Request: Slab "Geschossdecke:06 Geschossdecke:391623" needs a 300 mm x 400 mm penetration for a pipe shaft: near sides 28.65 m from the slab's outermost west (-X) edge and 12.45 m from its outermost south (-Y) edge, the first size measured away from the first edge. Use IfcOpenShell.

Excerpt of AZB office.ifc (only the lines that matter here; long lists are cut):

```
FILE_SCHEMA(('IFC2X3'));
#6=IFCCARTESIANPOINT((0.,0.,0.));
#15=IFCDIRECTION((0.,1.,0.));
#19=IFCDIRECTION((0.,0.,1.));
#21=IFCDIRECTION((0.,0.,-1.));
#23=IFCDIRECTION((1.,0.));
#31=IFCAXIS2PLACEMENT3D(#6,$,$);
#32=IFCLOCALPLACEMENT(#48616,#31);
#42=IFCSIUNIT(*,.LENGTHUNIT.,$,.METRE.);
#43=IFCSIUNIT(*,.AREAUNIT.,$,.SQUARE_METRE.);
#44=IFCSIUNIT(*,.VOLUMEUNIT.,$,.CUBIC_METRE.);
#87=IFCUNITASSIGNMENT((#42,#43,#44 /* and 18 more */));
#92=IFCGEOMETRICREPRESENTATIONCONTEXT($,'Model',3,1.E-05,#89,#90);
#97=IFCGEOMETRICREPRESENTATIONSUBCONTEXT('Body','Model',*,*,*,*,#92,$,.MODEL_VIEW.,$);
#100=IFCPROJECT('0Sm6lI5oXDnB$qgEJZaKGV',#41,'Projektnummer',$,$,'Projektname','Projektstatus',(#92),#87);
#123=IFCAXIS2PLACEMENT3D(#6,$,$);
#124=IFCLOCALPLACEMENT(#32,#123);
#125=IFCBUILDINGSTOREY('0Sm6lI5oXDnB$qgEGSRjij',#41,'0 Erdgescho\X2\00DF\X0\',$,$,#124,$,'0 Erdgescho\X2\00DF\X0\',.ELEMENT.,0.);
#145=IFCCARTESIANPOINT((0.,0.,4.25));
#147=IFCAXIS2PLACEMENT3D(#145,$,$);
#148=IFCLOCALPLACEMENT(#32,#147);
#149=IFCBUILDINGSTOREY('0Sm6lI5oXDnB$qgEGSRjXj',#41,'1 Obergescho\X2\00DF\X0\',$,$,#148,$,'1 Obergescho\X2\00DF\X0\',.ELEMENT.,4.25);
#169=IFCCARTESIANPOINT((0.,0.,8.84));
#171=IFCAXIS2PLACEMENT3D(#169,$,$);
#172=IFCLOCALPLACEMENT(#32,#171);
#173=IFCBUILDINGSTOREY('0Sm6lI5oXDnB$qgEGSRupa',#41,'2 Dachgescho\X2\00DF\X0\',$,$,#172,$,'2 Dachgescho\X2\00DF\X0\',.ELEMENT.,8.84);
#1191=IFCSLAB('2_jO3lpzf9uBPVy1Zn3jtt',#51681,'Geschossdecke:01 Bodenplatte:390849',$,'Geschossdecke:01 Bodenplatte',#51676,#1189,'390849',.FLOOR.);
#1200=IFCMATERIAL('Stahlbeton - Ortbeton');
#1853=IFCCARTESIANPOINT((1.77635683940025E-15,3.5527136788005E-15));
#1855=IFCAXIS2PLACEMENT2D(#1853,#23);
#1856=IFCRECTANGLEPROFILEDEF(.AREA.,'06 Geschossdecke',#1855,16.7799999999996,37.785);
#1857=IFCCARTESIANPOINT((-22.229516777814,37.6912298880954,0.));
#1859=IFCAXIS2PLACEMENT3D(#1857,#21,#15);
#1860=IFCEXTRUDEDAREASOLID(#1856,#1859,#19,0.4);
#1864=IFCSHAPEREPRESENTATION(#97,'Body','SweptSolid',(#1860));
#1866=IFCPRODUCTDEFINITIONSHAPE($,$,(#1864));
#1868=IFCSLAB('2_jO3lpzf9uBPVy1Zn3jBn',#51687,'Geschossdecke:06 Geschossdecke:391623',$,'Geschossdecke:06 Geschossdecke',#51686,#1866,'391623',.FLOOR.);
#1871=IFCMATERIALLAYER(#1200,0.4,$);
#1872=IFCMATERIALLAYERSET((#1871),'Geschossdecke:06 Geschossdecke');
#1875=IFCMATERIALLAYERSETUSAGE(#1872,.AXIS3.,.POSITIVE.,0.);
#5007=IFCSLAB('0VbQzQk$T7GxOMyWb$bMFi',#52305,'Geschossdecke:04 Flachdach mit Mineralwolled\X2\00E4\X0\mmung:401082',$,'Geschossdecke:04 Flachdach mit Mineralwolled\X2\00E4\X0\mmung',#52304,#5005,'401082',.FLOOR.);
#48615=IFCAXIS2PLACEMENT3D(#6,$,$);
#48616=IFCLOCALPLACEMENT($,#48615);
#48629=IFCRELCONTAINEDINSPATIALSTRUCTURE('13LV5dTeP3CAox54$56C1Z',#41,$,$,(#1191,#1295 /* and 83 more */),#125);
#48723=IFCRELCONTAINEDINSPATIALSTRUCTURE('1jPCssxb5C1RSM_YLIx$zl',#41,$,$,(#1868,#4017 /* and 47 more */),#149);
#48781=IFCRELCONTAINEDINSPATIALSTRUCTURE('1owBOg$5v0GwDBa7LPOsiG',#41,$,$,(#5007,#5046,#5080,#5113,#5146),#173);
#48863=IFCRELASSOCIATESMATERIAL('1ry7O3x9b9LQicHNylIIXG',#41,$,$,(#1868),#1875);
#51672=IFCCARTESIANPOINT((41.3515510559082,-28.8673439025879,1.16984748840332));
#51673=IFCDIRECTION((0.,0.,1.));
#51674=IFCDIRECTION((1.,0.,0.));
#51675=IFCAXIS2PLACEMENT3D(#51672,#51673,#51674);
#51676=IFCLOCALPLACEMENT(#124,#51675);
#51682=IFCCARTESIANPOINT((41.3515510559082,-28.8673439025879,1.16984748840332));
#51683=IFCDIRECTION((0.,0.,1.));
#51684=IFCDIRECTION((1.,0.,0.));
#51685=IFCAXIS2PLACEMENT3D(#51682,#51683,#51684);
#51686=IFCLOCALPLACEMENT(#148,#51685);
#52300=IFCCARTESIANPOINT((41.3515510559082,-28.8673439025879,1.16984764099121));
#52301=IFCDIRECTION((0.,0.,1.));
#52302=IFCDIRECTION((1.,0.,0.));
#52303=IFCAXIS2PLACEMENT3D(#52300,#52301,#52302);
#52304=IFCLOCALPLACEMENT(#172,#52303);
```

```python
import numpy as np
import ifcopenshell
import ifcopenshell.api.feature
import ifcopenshell.api.geometry
import ifcopenshell.api.root
import ifcopenshell.geom
import ifcopenshell.util.placement
import ifcopenshell.util.representation
import ifcopenshell.util.shape
import ifcopenshell.util.unit

model = ifcopenshell.open("AZB office.ifc")
unit_scale = ifcopenshell.util.unit.calculate_unit_scale(model)
settings = ifcopenshell.geom.settings()


def volume(element):
    """Net volume in cubic metres, openings subtracted."""
    shape = ifcopenshell.geom.create_shape(settings, element)
    return ifcopenshell.util.shape.get_volume(shape.geometry)


slab = model.by_guid("2_jO3lpzf9uBPVy1Zn3jBn")
before = volume(slab)

# Extent in the slab's own axes, in metres. The edges named are its -X and -Y sides.
slab_shape = ifcopenshell.geom.create_shape(settings, slab)
vertices = ifcopenshell.util.shape.get_vertices(slab_shape.geometry)
x_min, y_min, bottom = vertices.min(axis=0)
top = vertices[:, 2].max()

opening = ifcopenshell.api.root.create_entity(model, ifc_class="IfcOpeningElement", name="Pipe shaft opening")
context = ifcopenshell.util.representation.get_context(model, "Model", "Body", "MODEL_VIEW")
width, depth = 0.3, 0.4
outline = [(0.0, 0.0), (width, 0.0), (width, depth), (0.0, depth), (0.0, 0.0)]
# Overshoot both faces by 50 mm so the cut is clean.
shape = ifcopenshell.api.geometry.add_slab_representation(
    model, context=context, depth=top - bottom + 0.1, polyline=outline
)
ifcopenshell.api.geometry.assign_representation(model, product=opening, representation=shape)

matrix = ifcopenshell.util.placement.get_local_placement(slab.ObjectPlacement)
matrix[:, 3] = matrix @ np.append(np.array([x_min + 28.65, y_min + 12.45, bottom - 0.05]) / unit_scale, 1.0)
ifcopenshell.api.geometry.edit_object_placement(model, product=opening, matrix=matrix, is_si=False)
ifcopenshell.api.feature.add_feature(model, feature=opening, element=slab)

after = volume(slab)

print(f"slab volume {before:.3f} -> {after:.3f} m3")

model.write("AZB office-out.ifc")
```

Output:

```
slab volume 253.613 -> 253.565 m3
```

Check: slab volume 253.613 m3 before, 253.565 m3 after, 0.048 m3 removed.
